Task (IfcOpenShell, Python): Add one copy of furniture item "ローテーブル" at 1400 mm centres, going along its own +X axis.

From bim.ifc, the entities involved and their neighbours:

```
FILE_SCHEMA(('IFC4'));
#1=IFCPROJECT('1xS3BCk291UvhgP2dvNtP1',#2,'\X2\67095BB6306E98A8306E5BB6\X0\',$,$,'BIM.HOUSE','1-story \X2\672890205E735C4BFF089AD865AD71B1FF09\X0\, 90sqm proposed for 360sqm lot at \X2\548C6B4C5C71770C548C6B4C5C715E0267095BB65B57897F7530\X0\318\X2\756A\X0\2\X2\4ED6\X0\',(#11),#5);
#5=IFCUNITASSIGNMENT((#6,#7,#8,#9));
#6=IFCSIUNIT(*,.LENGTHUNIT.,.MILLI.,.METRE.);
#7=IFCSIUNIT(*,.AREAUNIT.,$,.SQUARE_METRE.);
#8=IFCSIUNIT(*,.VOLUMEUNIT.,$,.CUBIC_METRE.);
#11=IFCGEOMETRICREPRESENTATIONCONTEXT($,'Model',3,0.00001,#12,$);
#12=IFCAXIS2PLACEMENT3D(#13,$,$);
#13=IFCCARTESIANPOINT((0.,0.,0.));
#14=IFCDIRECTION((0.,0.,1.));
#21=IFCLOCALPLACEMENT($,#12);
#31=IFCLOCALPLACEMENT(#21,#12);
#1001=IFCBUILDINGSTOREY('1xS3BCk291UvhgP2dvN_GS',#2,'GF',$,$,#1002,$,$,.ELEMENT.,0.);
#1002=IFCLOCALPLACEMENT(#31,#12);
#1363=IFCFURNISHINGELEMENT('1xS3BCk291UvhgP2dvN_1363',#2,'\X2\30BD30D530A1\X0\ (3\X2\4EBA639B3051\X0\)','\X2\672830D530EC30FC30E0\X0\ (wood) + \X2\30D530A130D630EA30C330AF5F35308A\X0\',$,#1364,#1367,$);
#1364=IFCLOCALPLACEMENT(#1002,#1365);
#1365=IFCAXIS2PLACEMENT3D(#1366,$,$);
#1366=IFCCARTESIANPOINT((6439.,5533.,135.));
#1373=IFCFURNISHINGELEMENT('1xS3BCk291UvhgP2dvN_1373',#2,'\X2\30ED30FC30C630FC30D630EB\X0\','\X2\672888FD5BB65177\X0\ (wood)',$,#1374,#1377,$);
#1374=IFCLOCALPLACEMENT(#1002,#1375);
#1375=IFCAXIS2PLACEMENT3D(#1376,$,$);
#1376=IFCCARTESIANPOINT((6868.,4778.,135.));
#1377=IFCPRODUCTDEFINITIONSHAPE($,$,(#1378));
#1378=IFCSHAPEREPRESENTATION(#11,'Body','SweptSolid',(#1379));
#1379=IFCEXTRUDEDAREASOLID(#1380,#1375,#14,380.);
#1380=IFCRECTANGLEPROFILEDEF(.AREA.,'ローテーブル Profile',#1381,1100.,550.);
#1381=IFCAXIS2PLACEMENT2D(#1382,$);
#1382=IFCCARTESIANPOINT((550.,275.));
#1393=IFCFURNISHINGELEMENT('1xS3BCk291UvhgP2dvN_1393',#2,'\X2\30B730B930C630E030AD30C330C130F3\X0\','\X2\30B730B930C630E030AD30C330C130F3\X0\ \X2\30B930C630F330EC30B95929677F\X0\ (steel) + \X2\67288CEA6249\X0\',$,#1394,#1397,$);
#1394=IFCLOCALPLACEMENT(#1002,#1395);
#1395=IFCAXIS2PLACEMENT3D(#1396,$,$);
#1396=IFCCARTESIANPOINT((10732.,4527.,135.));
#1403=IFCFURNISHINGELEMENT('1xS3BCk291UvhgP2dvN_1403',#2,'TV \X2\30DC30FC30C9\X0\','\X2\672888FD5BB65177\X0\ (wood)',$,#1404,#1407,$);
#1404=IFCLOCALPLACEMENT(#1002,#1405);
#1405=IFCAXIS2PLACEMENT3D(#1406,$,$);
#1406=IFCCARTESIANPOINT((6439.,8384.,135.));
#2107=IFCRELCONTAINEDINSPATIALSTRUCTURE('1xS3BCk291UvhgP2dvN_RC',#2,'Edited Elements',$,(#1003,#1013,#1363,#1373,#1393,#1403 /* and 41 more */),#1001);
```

```python
import ifcopenshell
import ifcopenshell.api.geometry
import ifcopenshell.api.root
import ifcopenshell.util.element
import ifcopenshell.util.placement
import ifcopenshell.util.unit

model = ifcopenshell.open("bim.ifc")
unit_scale = ifcopenshell.util.unit.calculate_unit_scale(model)


def reuse_history(source, copy):
    """copy_class also copies each property set's owner history, people and application; keep the originals."""
    for rel in copy.IsDefinedBy:
        if rel.is_a("IfcRelDefinesByProperties") and (history := rel.RelatingPropertyDefinition.OwnerHistory):
            rel.RelatingPropertyDefinition.OwnerHistory = source.OwnerHistory
            ifcopenshell.util.element.remove_deep2(model, history)


source = model.by_guid("1xS3BCk291UvhgP2dvN_1373")
base = ifcopenshell.util.placement.get_local_placement(source.ObjectPlacement)
step = base[:3, 0] * 1.4 / unit_scale

for i in range(1, 2):
    copy = ifcopenshell.api.root.copy_class(model, product=source)
    copy.Representation = ifcopenshell.util.element.copy_deep(
        model, source.Representation, exclude=["IfcGeometricRepresentationContext", "IfcRepresentationMap"]
    )
    reuse_history(source, copy)
    matrix = base.copy()
    matrix[:3, 3] += i * step
    print("added at", matrix[:3, 3].round(3) + 0.0)
    ifcopenshell.api.geometry.edit_object_placement(model, product=copy, matrix=matrix, is_si=False)

model.write("bim_v2.ifc")
```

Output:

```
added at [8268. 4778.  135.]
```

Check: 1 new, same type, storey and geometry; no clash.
